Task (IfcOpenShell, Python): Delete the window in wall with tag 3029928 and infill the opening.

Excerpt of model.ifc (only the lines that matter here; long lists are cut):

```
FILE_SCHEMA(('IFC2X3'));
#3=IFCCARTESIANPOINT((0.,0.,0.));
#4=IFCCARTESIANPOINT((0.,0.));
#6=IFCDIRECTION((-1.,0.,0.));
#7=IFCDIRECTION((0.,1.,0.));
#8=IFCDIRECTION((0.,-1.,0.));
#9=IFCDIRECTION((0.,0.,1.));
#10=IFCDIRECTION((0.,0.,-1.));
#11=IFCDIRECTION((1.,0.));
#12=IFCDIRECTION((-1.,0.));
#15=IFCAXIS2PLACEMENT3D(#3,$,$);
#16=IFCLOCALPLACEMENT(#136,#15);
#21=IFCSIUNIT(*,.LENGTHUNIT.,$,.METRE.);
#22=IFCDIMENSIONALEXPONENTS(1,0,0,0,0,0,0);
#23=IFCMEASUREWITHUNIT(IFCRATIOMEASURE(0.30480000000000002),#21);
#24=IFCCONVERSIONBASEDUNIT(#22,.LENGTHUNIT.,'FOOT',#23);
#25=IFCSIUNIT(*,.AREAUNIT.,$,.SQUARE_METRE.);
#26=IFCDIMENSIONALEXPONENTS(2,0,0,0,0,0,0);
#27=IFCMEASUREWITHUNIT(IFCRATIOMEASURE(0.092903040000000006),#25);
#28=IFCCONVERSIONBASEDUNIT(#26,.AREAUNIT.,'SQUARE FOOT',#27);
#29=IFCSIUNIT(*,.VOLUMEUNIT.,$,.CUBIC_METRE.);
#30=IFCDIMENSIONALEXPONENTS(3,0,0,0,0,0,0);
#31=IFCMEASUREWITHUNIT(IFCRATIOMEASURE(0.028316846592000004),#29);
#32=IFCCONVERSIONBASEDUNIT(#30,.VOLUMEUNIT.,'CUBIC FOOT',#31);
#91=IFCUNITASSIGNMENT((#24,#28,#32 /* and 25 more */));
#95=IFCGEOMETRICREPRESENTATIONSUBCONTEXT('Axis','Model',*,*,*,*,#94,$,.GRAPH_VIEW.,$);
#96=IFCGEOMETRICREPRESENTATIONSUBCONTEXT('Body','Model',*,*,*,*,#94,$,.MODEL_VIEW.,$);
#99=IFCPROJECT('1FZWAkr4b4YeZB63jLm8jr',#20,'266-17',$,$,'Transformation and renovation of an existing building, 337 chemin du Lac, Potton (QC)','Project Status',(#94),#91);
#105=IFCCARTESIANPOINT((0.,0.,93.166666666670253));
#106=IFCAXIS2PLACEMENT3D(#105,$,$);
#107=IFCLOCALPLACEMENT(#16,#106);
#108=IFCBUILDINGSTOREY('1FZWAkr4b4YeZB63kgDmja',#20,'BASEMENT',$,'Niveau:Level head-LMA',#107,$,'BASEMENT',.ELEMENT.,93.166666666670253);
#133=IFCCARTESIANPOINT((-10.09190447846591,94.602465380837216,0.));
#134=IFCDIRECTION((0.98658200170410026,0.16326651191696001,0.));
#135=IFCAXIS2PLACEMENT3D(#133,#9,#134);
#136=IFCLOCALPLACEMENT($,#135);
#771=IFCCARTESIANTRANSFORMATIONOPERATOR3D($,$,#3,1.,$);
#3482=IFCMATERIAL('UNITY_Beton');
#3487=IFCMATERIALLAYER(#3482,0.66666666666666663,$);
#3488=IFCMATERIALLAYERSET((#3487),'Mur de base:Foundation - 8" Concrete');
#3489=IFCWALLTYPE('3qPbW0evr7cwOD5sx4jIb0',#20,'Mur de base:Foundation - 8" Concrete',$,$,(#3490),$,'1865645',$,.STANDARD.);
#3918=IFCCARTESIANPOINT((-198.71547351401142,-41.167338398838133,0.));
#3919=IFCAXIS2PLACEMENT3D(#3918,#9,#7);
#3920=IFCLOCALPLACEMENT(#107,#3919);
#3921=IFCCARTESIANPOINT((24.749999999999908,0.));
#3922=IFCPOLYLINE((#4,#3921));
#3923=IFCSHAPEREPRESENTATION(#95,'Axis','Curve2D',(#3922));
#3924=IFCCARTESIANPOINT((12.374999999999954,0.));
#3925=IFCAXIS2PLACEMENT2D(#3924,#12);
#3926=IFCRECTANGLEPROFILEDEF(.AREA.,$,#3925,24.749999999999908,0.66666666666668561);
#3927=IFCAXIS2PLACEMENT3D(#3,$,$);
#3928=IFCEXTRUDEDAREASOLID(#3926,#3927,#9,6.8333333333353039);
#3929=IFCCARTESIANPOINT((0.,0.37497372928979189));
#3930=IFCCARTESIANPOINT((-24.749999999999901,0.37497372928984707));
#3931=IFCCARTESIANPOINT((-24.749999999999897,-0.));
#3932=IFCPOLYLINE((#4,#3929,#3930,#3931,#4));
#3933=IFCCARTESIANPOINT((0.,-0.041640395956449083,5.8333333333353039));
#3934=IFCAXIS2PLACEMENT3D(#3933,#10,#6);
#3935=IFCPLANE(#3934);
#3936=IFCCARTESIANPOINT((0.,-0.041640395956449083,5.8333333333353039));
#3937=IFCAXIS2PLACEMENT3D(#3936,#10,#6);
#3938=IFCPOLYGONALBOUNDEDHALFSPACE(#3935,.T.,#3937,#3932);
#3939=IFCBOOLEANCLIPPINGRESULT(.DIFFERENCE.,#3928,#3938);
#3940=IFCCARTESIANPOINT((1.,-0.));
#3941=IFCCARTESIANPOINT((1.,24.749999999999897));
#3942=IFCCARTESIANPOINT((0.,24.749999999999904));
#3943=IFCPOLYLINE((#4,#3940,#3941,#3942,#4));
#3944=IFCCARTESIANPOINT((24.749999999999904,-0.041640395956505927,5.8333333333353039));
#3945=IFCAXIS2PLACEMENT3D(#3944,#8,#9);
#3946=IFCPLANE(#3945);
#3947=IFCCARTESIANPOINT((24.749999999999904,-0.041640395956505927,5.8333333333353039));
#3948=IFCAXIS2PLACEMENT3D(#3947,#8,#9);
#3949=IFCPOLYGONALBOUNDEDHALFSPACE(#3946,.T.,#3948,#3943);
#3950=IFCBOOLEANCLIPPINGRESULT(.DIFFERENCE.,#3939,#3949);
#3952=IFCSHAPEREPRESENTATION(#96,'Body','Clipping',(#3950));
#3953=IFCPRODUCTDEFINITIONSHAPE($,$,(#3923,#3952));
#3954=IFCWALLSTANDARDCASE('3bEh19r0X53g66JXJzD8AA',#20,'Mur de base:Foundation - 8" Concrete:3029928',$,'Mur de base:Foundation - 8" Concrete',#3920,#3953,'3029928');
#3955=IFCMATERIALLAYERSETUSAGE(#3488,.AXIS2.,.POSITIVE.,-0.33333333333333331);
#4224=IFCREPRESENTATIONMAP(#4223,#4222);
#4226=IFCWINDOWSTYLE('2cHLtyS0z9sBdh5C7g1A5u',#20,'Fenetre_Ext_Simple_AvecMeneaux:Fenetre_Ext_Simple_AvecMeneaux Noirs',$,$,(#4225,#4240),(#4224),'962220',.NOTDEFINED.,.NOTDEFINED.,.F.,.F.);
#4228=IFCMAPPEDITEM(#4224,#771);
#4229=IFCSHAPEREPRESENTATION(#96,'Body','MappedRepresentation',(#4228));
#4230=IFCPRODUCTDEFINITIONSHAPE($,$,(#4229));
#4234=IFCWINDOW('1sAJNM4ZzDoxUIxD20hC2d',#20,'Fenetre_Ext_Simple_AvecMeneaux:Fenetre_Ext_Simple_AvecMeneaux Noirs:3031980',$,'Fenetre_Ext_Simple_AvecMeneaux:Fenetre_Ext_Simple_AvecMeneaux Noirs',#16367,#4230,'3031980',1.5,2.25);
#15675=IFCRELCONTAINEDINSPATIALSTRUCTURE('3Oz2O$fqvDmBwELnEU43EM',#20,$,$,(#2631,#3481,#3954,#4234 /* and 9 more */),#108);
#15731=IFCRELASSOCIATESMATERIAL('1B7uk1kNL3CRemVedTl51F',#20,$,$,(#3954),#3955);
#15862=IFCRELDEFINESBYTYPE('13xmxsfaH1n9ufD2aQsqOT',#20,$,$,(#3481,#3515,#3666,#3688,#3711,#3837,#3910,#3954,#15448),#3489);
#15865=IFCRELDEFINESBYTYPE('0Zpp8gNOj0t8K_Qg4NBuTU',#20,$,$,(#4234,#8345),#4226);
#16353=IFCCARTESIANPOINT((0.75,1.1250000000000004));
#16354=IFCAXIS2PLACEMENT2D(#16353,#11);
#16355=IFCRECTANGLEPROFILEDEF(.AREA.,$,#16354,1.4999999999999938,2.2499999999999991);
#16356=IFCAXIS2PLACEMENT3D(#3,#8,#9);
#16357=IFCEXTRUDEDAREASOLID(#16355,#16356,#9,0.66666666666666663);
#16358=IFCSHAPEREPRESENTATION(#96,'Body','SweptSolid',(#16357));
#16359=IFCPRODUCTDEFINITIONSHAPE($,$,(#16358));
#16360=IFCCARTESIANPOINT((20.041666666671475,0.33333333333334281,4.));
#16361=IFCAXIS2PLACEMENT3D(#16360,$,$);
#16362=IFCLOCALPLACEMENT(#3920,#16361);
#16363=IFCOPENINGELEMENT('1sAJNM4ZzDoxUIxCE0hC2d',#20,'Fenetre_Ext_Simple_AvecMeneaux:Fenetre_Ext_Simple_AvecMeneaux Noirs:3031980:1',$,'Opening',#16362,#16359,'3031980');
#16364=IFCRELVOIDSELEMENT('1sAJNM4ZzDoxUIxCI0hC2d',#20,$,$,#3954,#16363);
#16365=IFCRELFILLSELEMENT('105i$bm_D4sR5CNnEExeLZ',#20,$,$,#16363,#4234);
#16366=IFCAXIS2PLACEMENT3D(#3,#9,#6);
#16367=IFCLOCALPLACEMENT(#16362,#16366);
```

```python
import ifcopenshell
import ifcopenshell.api.feature
import ifcopenshell.api.root
import ifcopenshell.geom
import ifcopenshell.util.shape

model = ifcopenshell.open("model.ifc")
settings = ifcopenshell.geom.settings()


def volume(element):
    """Net volume in cubic metres, openings subtracted."""
    shape = ifcopenshell.geom.create_shape(settings, element)
    return ifcopenshell.util.shape.get_volume(shape.geometry)


window = model.by_id(4234)
opening = window.FillsVoids[0].RelatingOpeningElement
wall = opening.VoidsElements[0].RelatingBuildingElement
before = volume(wall)

ifcopenshell.api.root.remove_product(model, product=window)
ifcopenshell.api.feature.remove_feature(model, feature=opening)

after = volume(wall)

print(f"wall volume {before:.3f} -> {after:.3f} m3")

model.write("model_edited.ifc")
```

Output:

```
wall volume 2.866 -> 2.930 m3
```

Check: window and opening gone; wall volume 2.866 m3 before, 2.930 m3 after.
